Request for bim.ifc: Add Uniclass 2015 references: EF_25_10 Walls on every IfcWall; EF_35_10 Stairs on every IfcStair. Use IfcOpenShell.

First a look at what the model holds.

```python
import ifcopenshell

model = ifcopenshell.open("bim.ifc")
print(model.schema)
print("classifications:", [c.Name for c in model.by_type("IfcClassification")])
for ifc_class in ("IfcDoor", "IfcRoof", "IfcStair", "IfcWall", "IfcWindow"):
    print(ifc_class, len(model.by_type(ifc_class)))
```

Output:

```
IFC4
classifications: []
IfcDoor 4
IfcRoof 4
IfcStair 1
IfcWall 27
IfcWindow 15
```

```python
import ifcopenshell
import ifcopenshell.api.classification

model = ifcopenshell.open("bim.ifc")

system = ifcopenshell.api.classification.add_classification(model, classification="Uniclass 2015")

codes = {
    "IfcWall": ("EF_25_10", "Walls"),
    "IfcStair": ("EF_35_10", "Stairs"),
}
for ifc_class, (code, name) in codes.items():
    products = model.by_type(ifc_class)
    ifcopenshell.api.classification.add_reference(
        model, products=products, classification=system, identification=code, name=name
    )
    print(code, len(products))

model.write("bim_updated.ifc")
```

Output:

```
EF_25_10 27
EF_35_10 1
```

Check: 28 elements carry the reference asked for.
